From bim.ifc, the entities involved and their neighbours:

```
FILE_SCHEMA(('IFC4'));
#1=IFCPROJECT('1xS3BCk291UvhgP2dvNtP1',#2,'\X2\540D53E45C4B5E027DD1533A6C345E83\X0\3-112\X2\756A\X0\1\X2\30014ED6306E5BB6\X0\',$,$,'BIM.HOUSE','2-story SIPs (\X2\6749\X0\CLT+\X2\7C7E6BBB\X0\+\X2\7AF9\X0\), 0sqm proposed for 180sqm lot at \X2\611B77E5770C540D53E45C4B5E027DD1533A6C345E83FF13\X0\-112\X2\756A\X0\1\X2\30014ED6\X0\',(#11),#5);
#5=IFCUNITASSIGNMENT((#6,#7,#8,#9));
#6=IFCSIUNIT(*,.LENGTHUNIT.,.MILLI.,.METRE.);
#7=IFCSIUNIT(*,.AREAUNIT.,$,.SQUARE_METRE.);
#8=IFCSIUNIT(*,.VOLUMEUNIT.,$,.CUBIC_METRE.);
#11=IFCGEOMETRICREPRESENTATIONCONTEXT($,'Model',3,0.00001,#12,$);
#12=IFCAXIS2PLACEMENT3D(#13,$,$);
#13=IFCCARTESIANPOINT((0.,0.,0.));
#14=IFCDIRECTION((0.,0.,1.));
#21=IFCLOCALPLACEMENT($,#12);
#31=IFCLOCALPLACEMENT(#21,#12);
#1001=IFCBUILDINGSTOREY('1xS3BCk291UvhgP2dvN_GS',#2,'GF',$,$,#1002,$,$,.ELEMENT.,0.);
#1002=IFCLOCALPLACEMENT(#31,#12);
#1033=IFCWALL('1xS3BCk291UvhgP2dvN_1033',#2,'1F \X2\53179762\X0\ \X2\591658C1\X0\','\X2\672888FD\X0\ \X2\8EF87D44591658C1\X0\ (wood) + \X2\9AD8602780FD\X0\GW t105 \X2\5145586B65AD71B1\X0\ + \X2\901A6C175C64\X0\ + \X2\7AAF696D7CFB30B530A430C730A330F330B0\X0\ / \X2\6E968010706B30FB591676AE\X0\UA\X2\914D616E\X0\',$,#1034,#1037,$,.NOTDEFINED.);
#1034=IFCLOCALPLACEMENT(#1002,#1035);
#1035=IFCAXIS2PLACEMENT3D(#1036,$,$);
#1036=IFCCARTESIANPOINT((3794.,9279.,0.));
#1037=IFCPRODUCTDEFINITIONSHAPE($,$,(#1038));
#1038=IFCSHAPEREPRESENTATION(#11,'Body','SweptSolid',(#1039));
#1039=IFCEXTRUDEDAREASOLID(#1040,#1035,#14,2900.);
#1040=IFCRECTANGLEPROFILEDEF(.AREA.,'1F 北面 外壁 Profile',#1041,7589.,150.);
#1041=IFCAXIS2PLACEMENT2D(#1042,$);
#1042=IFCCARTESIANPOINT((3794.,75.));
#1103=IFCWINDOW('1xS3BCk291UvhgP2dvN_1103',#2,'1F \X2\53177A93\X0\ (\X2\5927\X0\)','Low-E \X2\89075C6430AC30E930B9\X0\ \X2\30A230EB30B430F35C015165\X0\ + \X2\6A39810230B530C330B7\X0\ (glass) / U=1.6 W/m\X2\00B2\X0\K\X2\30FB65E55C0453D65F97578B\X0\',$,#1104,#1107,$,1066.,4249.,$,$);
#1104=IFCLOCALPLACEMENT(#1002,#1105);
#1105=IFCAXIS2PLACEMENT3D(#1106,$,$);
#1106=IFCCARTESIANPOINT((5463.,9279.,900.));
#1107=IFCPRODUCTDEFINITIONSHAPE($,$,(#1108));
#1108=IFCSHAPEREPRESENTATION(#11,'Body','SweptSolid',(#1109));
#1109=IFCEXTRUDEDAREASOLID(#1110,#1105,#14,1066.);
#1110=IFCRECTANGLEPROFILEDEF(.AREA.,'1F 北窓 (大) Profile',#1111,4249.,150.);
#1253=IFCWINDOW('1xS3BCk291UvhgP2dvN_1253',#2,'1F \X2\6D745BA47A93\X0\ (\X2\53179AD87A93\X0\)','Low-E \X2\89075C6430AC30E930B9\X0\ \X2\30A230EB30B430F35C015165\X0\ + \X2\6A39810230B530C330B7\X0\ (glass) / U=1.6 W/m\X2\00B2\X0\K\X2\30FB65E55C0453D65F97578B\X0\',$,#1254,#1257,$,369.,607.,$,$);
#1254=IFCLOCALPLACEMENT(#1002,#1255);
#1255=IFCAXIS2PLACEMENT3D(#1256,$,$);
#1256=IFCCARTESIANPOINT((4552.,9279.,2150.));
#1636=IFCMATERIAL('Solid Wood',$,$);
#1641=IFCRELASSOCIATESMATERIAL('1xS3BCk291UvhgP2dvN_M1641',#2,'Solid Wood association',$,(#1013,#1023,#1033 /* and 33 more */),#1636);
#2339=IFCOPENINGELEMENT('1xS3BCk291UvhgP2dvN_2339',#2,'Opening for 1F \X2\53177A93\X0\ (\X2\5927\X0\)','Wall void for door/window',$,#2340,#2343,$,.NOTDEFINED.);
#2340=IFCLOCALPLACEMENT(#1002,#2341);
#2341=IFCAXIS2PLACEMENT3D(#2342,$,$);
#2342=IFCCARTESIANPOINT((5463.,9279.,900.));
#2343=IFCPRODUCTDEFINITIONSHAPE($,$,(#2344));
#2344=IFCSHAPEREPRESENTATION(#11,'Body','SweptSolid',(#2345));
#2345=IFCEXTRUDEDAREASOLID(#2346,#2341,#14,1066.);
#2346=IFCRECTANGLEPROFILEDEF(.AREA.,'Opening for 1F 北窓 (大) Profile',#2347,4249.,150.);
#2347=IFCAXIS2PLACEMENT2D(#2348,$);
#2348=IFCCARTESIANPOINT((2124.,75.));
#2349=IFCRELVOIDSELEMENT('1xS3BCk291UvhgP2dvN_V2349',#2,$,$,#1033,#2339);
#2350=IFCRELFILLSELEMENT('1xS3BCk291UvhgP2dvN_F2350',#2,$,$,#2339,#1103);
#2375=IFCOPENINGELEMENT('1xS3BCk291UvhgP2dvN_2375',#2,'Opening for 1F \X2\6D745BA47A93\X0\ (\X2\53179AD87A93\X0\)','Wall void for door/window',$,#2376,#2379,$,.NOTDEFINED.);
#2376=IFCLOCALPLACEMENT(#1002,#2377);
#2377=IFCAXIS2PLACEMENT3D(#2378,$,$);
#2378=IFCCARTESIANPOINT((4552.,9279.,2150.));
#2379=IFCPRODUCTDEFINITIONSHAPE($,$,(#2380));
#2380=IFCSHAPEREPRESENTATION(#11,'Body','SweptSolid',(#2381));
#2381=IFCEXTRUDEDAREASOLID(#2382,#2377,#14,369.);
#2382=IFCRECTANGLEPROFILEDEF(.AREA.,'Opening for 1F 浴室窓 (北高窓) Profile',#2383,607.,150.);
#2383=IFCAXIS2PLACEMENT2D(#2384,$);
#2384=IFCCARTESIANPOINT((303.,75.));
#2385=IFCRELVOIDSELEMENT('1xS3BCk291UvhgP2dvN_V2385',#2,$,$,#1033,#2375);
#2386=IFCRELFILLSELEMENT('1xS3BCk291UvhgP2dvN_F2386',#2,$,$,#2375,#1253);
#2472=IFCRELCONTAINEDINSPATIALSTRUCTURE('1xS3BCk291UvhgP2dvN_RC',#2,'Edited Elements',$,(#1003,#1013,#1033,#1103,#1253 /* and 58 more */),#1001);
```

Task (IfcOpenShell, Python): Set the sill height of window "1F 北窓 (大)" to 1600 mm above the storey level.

```python
import numpy as np
import ifcopenshell
import ifcopenshell.api.geometry
import ifcopenshell.geom
import ifcopenshell.util.element
import ifcopenshell.util.placement
import ifcopenshell.util.shape
import ifcopenshell.util.unit

model = ifcopenshell.open("bim.ifc")
unit_scale = ifcopenshell.util.unit.calculate_unit_scale(model)

window = model.by_id(1103)
opening = window.FillsVoids[0].RelatingOpeningElement
storey = ifcopenshell.util.element.get_container(window, ifc_class="IfcBuildingStorey")
level = ifcopenshell.util.placement.get_local_placement(storey.ObjectPlacement)[2, 3]

# The opening's origin need not be at the sill, so measure its lowest point.
shape = ifcopenshell.geom.create_shape(ifcopenshell.geom.settings(), opening)
bottom = ifcopenshell.util.shape.get_shape_bottom_elevation(shape, shape.geometry) / unit_scale
dz = level + 1600.0 - bottom

shift = np.array([0.0, 0.0, dz])
# The window is not placed relative to its opening, so move both.
for product in (opening, window):
    matrix = ifcopenshell.util.placement.get_local_placement(product.ObjectPlacement)
    matrix[:3, 3] += shift
    ifcopenshell.api.geometry.edit_object_placement(model, product=product, matrix=matrix, is_si=False)

print(f"moved by {dz * unit_scale:+.3f} m")

model.write("bim-out.ifc")
```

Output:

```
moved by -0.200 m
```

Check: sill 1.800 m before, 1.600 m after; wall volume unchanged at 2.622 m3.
